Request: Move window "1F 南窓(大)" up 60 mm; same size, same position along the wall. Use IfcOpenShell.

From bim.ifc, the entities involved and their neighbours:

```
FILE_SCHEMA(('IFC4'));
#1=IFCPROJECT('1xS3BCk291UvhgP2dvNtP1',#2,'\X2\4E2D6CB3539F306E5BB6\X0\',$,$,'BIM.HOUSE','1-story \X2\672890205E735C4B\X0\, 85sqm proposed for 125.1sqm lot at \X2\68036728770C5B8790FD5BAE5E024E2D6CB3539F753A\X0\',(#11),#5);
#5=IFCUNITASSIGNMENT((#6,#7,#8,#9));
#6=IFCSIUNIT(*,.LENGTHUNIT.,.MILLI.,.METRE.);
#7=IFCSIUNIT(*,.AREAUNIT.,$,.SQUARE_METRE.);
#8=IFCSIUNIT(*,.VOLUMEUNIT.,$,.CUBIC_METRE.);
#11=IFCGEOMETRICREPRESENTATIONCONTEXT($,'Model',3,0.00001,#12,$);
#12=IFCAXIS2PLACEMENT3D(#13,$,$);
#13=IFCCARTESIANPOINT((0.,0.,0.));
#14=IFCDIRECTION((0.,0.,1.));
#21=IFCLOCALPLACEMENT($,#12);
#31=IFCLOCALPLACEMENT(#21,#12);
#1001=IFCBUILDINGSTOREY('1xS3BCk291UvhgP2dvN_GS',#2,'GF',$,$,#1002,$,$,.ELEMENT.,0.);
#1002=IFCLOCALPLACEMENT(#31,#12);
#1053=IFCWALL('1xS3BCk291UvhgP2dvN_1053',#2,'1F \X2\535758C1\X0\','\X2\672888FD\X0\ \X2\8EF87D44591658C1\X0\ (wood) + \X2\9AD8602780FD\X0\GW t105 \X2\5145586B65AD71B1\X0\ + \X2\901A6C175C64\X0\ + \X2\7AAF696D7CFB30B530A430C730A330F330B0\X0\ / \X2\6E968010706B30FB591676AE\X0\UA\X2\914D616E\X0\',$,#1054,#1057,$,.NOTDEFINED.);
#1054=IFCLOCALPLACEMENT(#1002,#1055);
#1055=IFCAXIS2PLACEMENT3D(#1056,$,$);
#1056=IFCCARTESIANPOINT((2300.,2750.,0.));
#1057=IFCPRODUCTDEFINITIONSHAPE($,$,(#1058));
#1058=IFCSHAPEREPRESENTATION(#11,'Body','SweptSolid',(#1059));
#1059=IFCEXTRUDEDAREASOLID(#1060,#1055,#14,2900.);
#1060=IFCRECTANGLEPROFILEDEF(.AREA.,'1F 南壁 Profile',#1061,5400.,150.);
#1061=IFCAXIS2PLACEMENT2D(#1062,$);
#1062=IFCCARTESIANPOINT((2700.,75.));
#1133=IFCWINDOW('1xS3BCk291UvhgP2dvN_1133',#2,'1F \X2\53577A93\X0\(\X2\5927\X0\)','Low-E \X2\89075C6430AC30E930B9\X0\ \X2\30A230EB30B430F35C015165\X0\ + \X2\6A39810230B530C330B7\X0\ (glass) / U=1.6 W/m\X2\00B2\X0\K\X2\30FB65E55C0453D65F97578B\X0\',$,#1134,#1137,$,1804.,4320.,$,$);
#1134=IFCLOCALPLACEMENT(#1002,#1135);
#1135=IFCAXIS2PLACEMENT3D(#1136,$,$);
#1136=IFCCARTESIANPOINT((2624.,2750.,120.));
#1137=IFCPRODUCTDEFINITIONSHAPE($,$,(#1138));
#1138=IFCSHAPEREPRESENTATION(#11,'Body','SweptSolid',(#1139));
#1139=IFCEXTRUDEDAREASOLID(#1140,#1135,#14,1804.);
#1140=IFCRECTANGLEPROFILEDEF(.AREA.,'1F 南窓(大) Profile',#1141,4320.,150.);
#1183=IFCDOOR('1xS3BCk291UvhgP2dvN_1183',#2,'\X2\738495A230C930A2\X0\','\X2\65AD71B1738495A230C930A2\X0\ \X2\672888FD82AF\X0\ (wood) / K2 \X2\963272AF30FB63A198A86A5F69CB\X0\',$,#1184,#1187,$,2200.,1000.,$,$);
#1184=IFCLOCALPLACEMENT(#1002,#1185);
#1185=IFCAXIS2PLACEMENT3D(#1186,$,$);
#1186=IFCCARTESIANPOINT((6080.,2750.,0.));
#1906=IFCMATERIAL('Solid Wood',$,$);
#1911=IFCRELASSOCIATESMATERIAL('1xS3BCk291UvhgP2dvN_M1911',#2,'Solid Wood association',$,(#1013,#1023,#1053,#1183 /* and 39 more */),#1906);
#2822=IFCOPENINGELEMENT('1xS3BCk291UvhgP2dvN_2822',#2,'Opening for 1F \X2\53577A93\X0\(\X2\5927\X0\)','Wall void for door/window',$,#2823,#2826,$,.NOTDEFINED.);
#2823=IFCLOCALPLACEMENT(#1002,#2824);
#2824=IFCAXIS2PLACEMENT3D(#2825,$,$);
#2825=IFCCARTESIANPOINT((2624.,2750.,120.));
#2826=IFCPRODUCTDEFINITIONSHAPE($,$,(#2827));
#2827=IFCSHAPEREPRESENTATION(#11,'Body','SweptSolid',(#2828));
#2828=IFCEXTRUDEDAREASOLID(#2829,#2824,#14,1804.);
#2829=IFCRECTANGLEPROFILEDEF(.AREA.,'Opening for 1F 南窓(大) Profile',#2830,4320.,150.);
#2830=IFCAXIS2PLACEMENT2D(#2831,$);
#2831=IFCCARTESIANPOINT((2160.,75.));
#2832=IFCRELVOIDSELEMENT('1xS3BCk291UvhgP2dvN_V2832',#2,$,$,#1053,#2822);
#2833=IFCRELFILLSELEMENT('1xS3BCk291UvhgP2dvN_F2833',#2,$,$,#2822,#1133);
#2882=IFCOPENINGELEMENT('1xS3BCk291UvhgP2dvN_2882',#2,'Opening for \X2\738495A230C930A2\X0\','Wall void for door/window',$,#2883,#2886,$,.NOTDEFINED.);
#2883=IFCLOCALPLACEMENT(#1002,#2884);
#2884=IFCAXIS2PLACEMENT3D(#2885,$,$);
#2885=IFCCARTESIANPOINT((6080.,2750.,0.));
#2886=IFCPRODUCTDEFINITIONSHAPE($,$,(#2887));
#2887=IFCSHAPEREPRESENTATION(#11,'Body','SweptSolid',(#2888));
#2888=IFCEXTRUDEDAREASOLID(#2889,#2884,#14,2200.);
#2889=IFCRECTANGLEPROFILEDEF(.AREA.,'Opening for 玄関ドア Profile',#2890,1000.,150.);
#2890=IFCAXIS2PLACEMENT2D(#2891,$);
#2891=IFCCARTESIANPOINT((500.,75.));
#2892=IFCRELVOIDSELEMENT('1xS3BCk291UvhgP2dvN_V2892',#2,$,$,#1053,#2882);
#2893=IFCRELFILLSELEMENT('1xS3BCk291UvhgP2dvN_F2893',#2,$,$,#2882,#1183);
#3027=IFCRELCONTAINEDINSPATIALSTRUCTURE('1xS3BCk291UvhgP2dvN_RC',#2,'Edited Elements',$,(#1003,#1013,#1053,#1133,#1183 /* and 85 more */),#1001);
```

```python
import numpy as np
import ifcopenshell
import ifcopenshell.api.geometry
import ifcopenshell.util.placement
import ifcopenshell.util.unit

model = ifcopenshell.open("bim.ifc")
unit_scale = ifcopenshell.util.unit.calculate_unit_scale(model)

window = model.by_id(1133)
opening = window.FillsVoids[0].RelatingOpeningElement
dz = 0.06 / unit_scale

shift = np.array([0.0, 0.0, dz])
# The window is not placed relative to its opening, so move both.
for product in (opening, window):
    matrix = ifcopenshell.util.placement.get_local_placement(product.ObjectPlacement)
    matrix[:3, 3] += shift
    ifcopenshell.api.geometry.edit_object_placement(model, product=product, matrix=matrix, is_si=False)

print(f"moved by {dz * unit_scale:+.3f} m")

model.write("bim_v2.ifc")
```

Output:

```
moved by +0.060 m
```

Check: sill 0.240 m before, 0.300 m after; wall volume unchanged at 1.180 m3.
